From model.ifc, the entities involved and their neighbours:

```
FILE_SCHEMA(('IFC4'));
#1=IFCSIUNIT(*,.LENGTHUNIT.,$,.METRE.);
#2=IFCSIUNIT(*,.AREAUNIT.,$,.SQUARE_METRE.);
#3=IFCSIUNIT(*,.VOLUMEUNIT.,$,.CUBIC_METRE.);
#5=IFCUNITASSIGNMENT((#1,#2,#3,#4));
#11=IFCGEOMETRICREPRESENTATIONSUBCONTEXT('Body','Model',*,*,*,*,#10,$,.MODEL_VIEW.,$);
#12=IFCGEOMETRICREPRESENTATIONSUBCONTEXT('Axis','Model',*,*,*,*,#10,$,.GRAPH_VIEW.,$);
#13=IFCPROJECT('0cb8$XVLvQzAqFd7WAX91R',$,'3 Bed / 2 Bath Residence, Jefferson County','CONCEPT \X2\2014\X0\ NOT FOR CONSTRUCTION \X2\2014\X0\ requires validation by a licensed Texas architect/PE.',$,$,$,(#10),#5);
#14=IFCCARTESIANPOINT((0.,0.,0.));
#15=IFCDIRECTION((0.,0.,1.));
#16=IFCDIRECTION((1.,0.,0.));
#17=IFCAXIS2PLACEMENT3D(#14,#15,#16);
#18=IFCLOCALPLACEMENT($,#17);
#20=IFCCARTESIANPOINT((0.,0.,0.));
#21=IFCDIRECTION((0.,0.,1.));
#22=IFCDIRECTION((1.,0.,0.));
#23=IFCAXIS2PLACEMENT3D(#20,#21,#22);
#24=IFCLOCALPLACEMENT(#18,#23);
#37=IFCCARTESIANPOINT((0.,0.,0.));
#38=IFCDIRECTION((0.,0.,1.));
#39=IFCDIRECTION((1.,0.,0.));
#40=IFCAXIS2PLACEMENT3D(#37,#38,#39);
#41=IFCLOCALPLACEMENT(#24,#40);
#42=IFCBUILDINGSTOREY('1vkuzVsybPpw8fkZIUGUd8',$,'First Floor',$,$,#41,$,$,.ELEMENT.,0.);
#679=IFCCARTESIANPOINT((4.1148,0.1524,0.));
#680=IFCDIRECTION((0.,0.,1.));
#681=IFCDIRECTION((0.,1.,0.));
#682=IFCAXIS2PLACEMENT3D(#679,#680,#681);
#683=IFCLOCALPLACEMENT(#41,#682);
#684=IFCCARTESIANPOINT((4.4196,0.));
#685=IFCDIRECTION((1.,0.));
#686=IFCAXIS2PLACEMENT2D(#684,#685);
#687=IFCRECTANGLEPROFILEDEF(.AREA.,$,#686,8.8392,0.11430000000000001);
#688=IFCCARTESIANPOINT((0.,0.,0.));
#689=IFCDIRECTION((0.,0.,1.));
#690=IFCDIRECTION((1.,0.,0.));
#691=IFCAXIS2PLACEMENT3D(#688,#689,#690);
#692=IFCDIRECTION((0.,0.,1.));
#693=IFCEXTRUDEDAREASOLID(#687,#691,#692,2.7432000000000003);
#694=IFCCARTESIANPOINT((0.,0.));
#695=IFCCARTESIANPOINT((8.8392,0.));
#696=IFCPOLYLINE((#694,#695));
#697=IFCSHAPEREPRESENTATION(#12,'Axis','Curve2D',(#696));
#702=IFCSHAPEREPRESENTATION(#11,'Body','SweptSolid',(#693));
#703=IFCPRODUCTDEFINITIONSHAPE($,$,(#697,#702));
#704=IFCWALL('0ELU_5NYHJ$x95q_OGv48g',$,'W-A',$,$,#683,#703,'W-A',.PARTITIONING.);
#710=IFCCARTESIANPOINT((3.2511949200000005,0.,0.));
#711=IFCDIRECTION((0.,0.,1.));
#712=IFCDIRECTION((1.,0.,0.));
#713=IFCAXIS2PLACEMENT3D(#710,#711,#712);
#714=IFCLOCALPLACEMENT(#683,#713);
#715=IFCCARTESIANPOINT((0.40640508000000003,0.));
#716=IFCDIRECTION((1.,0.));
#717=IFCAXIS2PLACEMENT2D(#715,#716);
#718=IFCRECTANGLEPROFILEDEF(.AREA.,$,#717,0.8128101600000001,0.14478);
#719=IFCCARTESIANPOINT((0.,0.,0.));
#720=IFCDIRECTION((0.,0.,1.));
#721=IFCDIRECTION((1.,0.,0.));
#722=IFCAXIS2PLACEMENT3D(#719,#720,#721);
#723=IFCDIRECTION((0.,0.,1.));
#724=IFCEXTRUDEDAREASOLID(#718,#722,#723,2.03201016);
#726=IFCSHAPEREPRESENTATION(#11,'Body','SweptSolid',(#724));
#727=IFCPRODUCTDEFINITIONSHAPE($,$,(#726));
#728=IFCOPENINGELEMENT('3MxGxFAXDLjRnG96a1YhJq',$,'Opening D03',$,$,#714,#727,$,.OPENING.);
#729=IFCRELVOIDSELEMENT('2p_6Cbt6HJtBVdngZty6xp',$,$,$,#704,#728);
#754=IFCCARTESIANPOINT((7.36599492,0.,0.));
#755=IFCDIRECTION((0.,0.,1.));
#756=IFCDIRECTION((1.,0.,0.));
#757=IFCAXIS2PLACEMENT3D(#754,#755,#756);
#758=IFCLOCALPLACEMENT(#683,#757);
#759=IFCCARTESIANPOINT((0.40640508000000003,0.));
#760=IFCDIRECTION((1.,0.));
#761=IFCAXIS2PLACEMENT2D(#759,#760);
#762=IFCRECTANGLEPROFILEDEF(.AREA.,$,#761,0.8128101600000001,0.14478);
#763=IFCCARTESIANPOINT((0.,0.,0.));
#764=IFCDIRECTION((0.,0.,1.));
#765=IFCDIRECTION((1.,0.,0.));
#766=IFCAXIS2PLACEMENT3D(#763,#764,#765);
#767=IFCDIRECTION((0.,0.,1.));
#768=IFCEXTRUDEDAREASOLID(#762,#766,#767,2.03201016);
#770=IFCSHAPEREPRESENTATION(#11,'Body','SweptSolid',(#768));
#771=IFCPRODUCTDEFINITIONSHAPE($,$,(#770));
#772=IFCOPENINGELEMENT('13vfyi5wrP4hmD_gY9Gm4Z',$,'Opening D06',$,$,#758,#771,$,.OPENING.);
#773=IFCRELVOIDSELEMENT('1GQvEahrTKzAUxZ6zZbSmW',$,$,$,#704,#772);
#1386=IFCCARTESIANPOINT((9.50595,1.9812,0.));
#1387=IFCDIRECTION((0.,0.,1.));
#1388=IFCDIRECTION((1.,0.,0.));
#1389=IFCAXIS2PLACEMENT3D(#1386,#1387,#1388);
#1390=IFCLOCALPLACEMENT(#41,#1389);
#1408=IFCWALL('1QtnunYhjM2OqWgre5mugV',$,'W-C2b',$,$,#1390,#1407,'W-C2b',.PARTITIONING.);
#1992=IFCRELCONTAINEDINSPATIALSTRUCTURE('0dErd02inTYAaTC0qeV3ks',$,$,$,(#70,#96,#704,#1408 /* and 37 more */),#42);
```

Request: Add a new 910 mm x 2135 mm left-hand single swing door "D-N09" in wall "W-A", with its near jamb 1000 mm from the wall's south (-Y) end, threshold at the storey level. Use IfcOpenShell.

```python
import numpy as np
import ifcopenshell
import ifcopenshell.api.feature
import ifcopenshell.api.geometry
import ifcopenshell.api.root
import ifcopenshell.api.spatial
import ifcopenshell.geom
import ifcopenshell.util.element
import ifcopenshell.util.placement
import ifcopenshell.util.representation
import ifcopenshell.util.shape
import ifcopenshell.util.unit

model = ifcopenshell.open("model.ifc")
unit_scale = ifcopenshell.util.unit.calculate_unit_scale(model)
settings = ifcopenshell.geom.settings()


def volume(element):
    """Net volume in cubic metres, openings subtracted."""
    shape = ifcopenshell.geom.create_shape(settings, element)
    return ifcopenshell.util.shape.get_volume(shape.geometry)


wall = model.by_guid("0ELU_5NYHJ$x95q_OGv48g")
storey = ifcopenshell.util.element.get_container(wall, ifc_class="IfcBuildingStorey")
context = ifcopenshell.util.representation.get_context(model, "Model", "Body", "MODEL_VIEW")
before = volume(wall)

width, height, from_end, sill = 0.91, 2.135, 1, 0.0  # metres

# The wall runs along its own X axis, and the end named is its -X end.
wall_shape = ifcopenshell.geom.create_shape(settings, wall)
x, y, z = ifcopenshell.util.shape.get_vertices(wall_shape.geometry).T
start = x.min() + from_end
face, thickness = float(y.min()), float(y.max() - y.min())
wall_matrix = ifcopenshell.util.placement.get_local_placement(wall.ObjectPlacement)
level = ifcopenshell.util.placement.get_local_placement(storey.ObjectPlacement)[2, 3]


def in_wall(x, y):
    """Placement at x, y metres in the wall's axes, at sill height."""
    matrix = wall_matrix.copy()
    matrix[:, 3] = wall_matrix @ np.array([x / unit_scale, y / unit_scale, 0.0, 1.0])
    matrix[2, 3] = level + sill / unit_scale
    return matrix


# Opening: a box that overshoots both wall faces by 50 mm.
opening = ifcopenshell.api.root.create_entity(model, ifc_class="IfcOpeningElement", predefined_type="OPENING")
box = ifcopenshell.api.geometry.add_wall_representation(
    model, context=context, length=width, height=height, thickness=thickness + 0.1
)
ifcopenshell.api.geometry.assign_representation(model, product=opening, representation=box)
ifcopenshell.api.geometry.edit_object_placement(model, product=opening, matrix=in_wall(start, face - 0.05), is_si=False)
ifcopenshell.api.feature.add_feature(model, feature=opening, element=wall)

door = ifcopenshell.api.root.create_entity(model, ifc_class="IfcDoor", name="D-N09", predefined_type="DOOR")
door.OverallWidth, door.OverallHeight = width / unit_scale, height / unit_scale
door.OperationType = "SINGLE_SWING_LEFT"
body = ifcopenshell.api.geometry.add_door_representation(
    model,
    context=context,
    overall_width=door.OverallWidth,
    overall_height=door.OverallHeight,
    operation_type="SINGLE_SWING_LEFT",
    lining_properties={"LiningDepth": thickness / unit_scale, "ThresholdDepth": thickness / unit_scale},
)
ifcopenshell.api.geometry.assign_representation(model, product=door, representation=body)
ifcopenshell.api.spatial.assign_container(model, products=[door], relating_structure=storey)
ifcopenshell.api.feature.add_filling(model, opening=opening, element=door)

# The lining spans the wall, so the door starts at the wall face.
ifcopenshell.api.geometry.edit_object_placement(model, product=door, matrix=in_wall(start, face), is_si=False)

after = volume(wall)

print(f"wall volume {before:.3f} -> {after:.3f} m3")

model.write("model-out.ifc")
```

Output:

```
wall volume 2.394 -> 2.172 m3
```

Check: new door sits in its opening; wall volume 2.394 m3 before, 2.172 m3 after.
